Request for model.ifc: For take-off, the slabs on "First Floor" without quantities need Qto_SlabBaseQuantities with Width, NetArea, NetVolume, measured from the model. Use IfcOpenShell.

First a look at what the model holds.

```python
import ifcopenshell
import ifcopenshell.util.element
import ifcopenshell.util.unit

model = ifcopenshell.open("model.ifc")
print(model.schema)
for unit_type in ("LENGTHUNIT", "AREAUNIT", "VOLUMEUNIT"):
    print(unit_type, ifcopenshell.util.unit.calculate_unit_scale(model, unit_type))
storey = next(s for s in model.by_type("IfcBuildingStorey") if s.Name == "First Floor")
slabs = [e for e in ifcopenshell.util.element.get_decomposition(storey) if e.is_a("IfcSlab")]
for e in sorted(slabs, key=lambda e: e.id()):
    print(e.id(), e.is_a(), e.Name, list(ifcopenshell.util.element.get_psets(e, qtos_only=True)), sep=" | ")
```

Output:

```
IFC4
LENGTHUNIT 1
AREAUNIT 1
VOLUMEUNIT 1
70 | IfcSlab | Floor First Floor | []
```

```python
import ifcopenshell
import ifcopenshell.api.pset
import ifcopenshell.geom
import ifcopenshell.util.element
import ifcopenshell.util.shape
import ifcopenshell.util.unit

model = ifcopenshell.open("model.ifc")
unit_scale = ifcopenshell.util.unit.calculate_unit_scale(model)
area_scale = ifcopenshell.util.unit.calculate_unit_scale(model, "AREAUNIT")
volume_scale = ifcopenshell.util.unit.calculate_unit_scale(model, "VOLUMEUNIT")
settings = ifcopenshell.geom.settings()

storey = next(s for s in model.by_type("IfcBuildingStorey") if s.Name == "First Floor")
slabs = [e for e in ifcopenshell.util.element.get_decomposition(storey) if e.is_a("IfcSlab")]

for e in sorted(slabs, key=lambda e: e.id()):
    if ifcopenshell.util.element.get_psets(e, qtos_only=True, should_inherit=False):
        continue
    # Geometry comes back in metres, in the element's own axes.
    shape = ifcopenshell.geom.create_shape(settings, e)
    values = {
        "Width": ifcopenshell.util.shape.get_z(shape.geometry) / unit_scale,
        "NetArea": ifcopenshell.util.shape.get_footprint_area(shape.geometry) / area_scale,
        "NetVolume": ifcopenshell.util.shape.get_volume(shape.geometry) / volume_scale,
    }
    qto = ifcopenshell.api.pset.add_qto(model, product=e, name="Qto_SlabBaseQuantities")
    ifcopenshell.api.pset.edit_qto(model, qto=qto, properties=values)
    print(e.id(), {k: round(v, 3) for k, v in values.items()})

model.write("model_edited.ifc")
```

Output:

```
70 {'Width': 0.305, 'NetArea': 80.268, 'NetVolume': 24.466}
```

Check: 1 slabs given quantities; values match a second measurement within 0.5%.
